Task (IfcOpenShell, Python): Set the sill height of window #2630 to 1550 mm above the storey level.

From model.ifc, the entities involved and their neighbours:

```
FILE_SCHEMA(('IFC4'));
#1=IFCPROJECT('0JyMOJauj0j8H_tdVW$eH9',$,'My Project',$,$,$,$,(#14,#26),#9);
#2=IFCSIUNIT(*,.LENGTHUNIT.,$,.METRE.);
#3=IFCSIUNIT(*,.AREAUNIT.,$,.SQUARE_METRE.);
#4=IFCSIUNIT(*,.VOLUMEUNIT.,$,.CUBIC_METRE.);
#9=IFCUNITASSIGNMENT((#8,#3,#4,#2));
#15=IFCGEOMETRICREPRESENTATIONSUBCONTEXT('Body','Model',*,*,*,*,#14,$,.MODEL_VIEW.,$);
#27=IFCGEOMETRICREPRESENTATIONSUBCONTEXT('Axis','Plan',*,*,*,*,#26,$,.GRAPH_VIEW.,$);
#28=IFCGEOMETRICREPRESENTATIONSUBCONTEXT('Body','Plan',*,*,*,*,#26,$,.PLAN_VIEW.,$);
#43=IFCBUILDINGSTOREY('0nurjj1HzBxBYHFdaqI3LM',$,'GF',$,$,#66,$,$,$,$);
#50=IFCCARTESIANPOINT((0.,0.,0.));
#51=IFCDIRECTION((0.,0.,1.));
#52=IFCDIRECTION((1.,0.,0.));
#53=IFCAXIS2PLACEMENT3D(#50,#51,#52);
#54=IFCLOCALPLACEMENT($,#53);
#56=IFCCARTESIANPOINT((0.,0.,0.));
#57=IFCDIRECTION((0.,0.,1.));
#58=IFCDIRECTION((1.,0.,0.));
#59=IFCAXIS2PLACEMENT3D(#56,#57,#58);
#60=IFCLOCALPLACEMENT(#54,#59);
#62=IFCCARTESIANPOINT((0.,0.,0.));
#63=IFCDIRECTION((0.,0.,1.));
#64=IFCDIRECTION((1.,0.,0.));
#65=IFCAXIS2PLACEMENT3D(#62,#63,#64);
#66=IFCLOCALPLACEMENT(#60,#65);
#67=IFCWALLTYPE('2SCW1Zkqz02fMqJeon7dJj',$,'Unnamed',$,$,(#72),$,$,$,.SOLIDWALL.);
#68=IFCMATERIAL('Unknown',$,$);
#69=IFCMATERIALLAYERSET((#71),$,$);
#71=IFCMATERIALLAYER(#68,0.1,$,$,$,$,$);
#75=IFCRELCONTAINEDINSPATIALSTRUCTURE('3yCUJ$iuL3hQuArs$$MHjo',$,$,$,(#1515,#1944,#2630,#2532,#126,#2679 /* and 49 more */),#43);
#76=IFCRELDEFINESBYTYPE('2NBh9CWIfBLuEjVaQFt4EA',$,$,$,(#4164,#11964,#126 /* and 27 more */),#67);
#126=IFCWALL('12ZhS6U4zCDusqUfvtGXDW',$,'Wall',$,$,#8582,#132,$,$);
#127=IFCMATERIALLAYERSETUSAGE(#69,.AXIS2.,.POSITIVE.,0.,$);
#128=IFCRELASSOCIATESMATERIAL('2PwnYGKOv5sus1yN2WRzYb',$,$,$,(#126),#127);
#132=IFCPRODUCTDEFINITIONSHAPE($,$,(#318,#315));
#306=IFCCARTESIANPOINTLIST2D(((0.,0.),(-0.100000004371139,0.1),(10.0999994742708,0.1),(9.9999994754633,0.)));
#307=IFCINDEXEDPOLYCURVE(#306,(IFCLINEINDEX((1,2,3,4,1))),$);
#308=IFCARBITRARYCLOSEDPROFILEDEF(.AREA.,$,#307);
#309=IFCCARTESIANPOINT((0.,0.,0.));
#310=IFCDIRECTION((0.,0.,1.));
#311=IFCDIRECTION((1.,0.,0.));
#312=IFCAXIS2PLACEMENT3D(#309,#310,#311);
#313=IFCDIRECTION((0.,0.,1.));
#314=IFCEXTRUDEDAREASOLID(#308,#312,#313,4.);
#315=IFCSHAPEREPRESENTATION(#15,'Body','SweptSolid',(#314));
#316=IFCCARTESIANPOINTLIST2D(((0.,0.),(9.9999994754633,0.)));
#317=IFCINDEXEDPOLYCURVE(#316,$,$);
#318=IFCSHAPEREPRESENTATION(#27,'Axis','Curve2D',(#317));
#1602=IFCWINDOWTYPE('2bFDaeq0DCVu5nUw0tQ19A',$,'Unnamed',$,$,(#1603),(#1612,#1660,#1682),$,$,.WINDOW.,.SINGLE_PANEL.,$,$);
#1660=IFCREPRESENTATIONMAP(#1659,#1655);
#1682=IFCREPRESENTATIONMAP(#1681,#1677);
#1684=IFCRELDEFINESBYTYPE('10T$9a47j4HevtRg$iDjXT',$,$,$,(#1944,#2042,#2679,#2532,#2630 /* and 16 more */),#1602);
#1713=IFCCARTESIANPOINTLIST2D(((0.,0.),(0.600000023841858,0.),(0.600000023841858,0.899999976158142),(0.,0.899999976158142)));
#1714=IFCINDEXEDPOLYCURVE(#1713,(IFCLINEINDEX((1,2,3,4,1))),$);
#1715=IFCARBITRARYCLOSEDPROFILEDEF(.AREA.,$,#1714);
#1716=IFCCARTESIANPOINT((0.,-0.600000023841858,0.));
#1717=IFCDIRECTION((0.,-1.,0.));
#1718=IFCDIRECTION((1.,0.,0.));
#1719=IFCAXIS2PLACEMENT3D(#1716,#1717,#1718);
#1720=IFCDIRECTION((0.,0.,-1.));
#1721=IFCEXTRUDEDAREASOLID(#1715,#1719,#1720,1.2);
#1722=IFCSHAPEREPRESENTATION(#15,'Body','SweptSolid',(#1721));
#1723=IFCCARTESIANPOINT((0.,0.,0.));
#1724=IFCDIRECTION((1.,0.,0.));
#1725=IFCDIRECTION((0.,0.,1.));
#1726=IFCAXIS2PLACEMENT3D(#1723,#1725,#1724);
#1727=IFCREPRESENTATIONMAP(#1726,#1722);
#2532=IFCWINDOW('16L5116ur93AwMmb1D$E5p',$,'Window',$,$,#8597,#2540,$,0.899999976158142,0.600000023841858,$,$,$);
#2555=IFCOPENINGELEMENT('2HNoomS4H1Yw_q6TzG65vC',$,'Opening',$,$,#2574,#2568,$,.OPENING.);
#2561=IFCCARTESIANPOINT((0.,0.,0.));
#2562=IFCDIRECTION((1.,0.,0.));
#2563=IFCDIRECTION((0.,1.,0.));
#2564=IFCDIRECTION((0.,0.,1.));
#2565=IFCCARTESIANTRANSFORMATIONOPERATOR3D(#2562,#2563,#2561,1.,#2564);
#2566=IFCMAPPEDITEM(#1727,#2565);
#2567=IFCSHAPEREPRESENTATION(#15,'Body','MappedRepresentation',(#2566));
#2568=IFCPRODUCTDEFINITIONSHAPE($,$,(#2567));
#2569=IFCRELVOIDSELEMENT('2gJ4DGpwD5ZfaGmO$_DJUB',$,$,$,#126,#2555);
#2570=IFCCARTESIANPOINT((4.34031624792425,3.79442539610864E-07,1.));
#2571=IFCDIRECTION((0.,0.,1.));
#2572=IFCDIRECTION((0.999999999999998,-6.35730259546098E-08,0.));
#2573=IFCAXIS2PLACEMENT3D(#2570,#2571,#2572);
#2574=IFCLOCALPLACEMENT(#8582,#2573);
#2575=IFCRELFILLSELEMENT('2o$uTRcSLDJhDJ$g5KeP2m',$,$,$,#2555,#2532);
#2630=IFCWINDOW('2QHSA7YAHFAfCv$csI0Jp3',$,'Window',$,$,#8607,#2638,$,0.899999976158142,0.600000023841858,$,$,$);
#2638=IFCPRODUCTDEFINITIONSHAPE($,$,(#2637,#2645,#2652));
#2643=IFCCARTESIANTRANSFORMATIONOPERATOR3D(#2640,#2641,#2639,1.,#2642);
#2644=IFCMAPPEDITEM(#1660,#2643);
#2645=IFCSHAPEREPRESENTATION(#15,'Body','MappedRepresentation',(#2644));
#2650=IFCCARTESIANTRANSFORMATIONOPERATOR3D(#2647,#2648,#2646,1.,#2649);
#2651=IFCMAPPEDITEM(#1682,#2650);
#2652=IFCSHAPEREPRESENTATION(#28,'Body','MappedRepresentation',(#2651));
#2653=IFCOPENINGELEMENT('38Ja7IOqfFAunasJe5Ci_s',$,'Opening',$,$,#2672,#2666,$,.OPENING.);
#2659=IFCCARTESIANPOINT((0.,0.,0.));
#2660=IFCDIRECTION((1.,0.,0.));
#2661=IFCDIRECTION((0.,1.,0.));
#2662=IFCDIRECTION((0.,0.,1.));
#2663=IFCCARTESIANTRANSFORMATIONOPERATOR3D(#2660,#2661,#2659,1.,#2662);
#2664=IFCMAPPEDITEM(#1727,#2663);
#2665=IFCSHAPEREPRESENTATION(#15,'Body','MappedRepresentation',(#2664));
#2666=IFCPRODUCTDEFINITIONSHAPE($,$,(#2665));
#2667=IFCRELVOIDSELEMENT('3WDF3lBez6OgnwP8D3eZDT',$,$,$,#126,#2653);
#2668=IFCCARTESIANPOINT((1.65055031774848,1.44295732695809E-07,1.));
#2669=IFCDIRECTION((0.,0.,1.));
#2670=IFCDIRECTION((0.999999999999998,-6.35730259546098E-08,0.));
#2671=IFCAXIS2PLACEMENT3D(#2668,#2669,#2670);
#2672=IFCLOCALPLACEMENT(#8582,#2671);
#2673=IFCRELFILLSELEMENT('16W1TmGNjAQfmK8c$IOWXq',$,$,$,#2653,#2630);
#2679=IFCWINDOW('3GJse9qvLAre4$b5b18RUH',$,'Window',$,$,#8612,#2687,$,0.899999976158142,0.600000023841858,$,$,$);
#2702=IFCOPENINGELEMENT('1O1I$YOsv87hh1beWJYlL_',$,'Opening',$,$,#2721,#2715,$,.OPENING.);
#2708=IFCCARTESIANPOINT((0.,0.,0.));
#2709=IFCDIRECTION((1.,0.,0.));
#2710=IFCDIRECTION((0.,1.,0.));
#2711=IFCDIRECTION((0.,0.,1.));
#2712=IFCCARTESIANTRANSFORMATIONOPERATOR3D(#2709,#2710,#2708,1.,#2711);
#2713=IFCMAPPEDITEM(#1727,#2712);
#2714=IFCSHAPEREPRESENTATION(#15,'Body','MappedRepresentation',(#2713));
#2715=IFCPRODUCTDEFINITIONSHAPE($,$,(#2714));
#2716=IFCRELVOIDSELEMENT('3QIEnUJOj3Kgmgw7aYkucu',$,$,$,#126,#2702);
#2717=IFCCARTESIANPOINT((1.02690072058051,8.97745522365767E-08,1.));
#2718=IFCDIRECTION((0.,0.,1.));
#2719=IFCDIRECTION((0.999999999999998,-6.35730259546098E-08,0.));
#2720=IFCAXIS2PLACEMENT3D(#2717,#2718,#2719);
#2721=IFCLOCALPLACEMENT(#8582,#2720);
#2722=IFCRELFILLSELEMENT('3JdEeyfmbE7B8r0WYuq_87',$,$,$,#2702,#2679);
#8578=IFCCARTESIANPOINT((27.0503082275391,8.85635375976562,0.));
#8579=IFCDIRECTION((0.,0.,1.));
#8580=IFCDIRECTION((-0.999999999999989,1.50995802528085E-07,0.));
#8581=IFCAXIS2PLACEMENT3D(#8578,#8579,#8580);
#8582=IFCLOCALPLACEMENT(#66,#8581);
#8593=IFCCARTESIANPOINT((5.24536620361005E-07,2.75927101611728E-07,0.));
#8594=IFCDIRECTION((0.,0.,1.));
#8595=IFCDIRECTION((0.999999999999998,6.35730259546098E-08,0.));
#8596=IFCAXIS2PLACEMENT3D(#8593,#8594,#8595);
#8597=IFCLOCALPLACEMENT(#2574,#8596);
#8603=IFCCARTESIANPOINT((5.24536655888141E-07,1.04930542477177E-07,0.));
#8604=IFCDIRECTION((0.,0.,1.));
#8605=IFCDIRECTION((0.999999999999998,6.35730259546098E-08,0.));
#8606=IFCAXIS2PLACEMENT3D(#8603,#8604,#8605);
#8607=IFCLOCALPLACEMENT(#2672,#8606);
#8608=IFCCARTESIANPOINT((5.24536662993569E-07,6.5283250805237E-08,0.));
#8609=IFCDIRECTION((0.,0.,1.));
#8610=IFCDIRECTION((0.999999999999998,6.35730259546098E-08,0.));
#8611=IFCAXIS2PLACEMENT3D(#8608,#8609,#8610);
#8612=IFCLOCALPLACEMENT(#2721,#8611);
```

```python
import numpy as np
import ifcopenshell
import ifcopenshell.api.geometry
import ifcopenshell.geom
import ifcopenshell.util.element
import ifcopenshell.util.placement
import ifcopenshell.util.shape
import ifcopenshell.util.unit

model = ifcopenshell.open("model.ifc")
unit_scale = ifcopenshell.util.unit.calculate_unit_scale(model)

window = model.by_id(2630)
opening = window.FillsVoids[0].RelatingOpeningElement
storey = ifcopenshell.util.element.get_container(window, ifc_class="IfcBuildingStorey")
level = ifcopenshell.util.placement.get_local_placement(storey.ObjectPlacement)[2, 3]

# The opening's origin need not be at the sill, so measure its lowest point.
shape = ifcopenshell.geom.create_shape(ifcopenshell.geom.settings(), opening)
bottom = ifcopenshell.util.shape.get_shape_bottom_elevation(shape, shape.geometry) / unit_scale
dz = level + 1.55 / unit_scale - bottom

shift = np.array([0.0, 0.0, dz])
# The window is placed relative to its opening, so it follows when the opening moves.
matrix = ifcopenshell.util.placement.get_local_placement(opening.ObjectPlacement)
matrix[:3, 3] += shift
ifcopenshell.api.geometry.edit_object_placement(
    model, product=opening, matrix=matrix, is_si=False, should_transform_children=True
)

print(f"moved by {dz * unit_scale:+.3f} m")

model.write("model-out.ifc")
```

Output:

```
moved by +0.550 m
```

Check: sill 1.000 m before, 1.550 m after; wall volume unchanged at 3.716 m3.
